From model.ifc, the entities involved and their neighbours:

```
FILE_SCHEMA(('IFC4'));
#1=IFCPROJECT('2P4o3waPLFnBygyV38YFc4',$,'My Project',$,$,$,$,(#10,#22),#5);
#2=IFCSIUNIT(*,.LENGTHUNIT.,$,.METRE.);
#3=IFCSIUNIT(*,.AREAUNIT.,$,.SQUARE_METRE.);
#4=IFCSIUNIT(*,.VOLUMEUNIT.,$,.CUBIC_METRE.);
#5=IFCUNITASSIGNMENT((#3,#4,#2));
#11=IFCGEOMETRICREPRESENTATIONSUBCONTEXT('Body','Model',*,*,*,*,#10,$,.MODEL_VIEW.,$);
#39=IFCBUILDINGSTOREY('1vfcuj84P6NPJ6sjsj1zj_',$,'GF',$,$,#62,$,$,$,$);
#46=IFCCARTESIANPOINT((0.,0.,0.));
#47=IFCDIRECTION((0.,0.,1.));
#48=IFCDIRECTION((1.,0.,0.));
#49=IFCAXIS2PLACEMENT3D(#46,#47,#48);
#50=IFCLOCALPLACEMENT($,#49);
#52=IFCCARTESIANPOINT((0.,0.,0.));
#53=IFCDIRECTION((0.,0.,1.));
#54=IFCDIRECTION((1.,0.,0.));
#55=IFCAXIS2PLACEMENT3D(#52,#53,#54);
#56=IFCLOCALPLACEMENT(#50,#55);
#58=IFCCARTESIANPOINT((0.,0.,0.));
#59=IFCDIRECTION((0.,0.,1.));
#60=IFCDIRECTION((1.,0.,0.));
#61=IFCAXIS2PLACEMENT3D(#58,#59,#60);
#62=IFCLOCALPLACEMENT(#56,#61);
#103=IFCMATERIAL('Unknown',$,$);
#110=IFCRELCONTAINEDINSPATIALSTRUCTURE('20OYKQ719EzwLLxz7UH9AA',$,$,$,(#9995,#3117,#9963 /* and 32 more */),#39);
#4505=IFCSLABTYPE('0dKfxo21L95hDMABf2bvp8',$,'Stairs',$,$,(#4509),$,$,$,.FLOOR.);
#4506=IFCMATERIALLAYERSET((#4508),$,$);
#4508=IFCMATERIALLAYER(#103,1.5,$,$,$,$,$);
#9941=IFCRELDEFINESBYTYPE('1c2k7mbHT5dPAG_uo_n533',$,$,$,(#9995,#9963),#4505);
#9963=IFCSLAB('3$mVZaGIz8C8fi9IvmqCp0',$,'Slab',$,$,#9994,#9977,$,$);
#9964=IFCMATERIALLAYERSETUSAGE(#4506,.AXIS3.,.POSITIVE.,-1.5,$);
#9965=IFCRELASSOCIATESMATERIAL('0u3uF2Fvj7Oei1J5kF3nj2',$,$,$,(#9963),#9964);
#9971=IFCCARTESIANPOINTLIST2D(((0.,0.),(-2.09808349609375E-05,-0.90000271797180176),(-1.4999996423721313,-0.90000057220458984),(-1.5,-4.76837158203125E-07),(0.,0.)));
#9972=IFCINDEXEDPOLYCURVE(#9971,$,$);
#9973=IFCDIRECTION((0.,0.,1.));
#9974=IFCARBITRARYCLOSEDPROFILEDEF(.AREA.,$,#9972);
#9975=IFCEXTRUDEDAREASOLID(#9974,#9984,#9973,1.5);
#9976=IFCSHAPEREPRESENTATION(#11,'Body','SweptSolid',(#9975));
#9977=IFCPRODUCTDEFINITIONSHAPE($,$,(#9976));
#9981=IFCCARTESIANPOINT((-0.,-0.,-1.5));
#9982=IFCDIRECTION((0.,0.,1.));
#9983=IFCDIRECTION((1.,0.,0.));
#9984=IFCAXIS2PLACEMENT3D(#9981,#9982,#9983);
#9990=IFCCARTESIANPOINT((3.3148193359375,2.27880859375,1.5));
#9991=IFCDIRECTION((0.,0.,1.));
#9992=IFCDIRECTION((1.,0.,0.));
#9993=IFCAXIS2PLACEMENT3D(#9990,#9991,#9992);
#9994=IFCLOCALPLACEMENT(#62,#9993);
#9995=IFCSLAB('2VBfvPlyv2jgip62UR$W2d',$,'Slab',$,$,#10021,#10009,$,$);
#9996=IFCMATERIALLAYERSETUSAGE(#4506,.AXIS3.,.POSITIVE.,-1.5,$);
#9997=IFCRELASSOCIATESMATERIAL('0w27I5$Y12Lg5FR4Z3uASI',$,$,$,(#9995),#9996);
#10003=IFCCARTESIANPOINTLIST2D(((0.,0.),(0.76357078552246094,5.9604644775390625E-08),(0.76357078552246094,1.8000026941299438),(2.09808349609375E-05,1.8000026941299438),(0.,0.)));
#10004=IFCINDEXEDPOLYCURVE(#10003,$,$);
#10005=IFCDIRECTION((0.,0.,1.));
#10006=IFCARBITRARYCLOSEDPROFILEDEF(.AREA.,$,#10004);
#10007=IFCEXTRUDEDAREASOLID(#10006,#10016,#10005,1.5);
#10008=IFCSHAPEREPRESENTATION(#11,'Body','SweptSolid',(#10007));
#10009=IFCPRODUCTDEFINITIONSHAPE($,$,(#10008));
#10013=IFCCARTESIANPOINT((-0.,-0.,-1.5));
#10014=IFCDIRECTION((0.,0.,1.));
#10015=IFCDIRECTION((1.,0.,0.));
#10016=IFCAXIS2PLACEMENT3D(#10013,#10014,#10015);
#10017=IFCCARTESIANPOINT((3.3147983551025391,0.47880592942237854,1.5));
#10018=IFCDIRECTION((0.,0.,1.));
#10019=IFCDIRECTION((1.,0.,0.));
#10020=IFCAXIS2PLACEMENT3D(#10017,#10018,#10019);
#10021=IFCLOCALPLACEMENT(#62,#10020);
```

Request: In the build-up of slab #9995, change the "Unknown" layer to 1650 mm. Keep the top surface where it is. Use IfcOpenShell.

```python
import ifcopenshell
import ifcopenshell.util.element
import ifcopenshell.util.representation
import ifcopenshell.util.unit

model = ifcopenshell.open("model.ifc")
unit_scale = ifcopenshell.util.unit.calculate_unit_scale(model)

layer_set = model.by_id(4506)
layer = next(l for l in layer_set.MaterialLayers if l.Material and l.Material.Name == "Unknown")
change = 1.65 / unit_scale - layer.LayerThickness
layer.LayerThickness += change

# The layer set is shared, so every slab that uses it gets the new thickness.
slabs = [e for e in ifcopenshell.util.element.get_elements_by_material(model, layer_set) if e.is_a("IfcSlab")]
for slab in sorted(slabs, key=lambda e: e.id()):
    body = ifcopenshell.util.representation.get_representation(slab, "Model", "Body")
    solid = body.Items[0]
    old_depth = solid.Depth
    solid.Depth += change
    # Extruded upwards: lower the start of the extrusion so the top stays.
    x, y, z = solid.Position.Location.Coordinates
    solid.Position.Location = model.createIfcCartesianPoint((x, y, z - change))
    print(slab.id(), f"{old_depth:g} -> {solid.Depth:g}")

# The layers are counted up from the underside, which has moved.
for usage in {ifcopenshell.util.element.get_material(slab) for slab in slabs}:
    usage.OffsetFromReferenceLine -= change

model.write("model_rev.ifc")
```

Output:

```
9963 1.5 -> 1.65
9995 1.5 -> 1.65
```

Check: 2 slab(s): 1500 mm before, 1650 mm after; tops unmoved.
